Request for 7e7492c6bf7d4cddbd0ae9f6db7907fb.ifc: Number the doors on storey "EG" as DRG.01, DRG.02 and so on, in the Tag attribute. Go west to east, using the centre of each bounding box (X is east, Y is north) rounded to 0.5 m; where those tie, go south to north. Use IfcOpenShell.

First a look at what the model holds.

```python
import ifcopenshell
import ifcopenshell.util.element
import ifcopenshell.util.placement

model = ifcopenshell.open("7e7492c6bf7d4cddbd0ae9f6db7907fb.ifc")
print(model.schema)
storey = next(s for s in model.by_type("IfcBuildingStorey") if s.Name == "EG")
doors = [e for e in ifcopenshell.util.element.get_decomposition(storey) if e.is_a("IfcDoor")]
for e in sorted(doors, key=lambda e: e.id()):
    origin = ifcopenshell.util.placement.get_local_placement(e.ObjectPlacement)[:3, 3]
    print(e.id(), e.Tag, e.Name, origin.round(2) + 0.0, sep=" | ")
```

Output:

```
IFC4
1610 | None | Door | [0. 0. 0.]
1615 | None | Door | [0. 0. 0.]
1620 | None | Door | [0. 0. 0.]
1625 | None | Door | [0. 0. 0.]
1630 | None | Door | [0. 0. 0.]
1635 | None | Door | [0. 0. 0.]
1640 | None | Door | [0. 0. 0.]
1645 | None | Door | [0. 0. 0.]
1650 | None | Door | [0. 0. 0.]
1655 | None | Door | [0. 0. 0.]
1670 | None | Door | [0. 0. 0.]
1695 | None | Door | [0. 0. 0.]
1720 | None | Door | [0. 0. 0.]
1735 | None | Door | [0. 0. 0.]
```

```python
import ifcopenshell
import ifcopenshell.geom
import ifcopenshell.util.element
import ifcopenshell.util.shape

model = ifcopenshell.open("7e7492c6bf7d4cddbd0ae9f6db7907fb.ifc")
settings = ifcopenshell.geom.settings()
settings.set("use-world-coords", True)


def centre(element):
    shape = ifcopenshell.geom.create_shape(settings, element)
    return ifcopenshell.util.shape.get_bbox_centroid(shape.geometry)


storey = next(s for s in model.by_type("IfcBuildingStorey") if s.Name == "EG")
doors = [e for e in ifcopenshell.util.element.get_decomposition(storey) if e.is_a("IfcDoor")]

# Insertion points can sit at a corner or the storey origin, so sort by the geometry (in metres).
centres = {e: centre(e) for e in doors}
doors.sort(key=lambda e: (round(centres[e][0] / 0.5), centres[e][1]))

for i, e in enumerate(doors, start=1):
    number = f"DRG.{i:02d}"
    e.Tag = number
    print(e.id(), number)

model.write("7e7492c6bf7d4cddbd0ae9f6db7907fb-out.ifc")
```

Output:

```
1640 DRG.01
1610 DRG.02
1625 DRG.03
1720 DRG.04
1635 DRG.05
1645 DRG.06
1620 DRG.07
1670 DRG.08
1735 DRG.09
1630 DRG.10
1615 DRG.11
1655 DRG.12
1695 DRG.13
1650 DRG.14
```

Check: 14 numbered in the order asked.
